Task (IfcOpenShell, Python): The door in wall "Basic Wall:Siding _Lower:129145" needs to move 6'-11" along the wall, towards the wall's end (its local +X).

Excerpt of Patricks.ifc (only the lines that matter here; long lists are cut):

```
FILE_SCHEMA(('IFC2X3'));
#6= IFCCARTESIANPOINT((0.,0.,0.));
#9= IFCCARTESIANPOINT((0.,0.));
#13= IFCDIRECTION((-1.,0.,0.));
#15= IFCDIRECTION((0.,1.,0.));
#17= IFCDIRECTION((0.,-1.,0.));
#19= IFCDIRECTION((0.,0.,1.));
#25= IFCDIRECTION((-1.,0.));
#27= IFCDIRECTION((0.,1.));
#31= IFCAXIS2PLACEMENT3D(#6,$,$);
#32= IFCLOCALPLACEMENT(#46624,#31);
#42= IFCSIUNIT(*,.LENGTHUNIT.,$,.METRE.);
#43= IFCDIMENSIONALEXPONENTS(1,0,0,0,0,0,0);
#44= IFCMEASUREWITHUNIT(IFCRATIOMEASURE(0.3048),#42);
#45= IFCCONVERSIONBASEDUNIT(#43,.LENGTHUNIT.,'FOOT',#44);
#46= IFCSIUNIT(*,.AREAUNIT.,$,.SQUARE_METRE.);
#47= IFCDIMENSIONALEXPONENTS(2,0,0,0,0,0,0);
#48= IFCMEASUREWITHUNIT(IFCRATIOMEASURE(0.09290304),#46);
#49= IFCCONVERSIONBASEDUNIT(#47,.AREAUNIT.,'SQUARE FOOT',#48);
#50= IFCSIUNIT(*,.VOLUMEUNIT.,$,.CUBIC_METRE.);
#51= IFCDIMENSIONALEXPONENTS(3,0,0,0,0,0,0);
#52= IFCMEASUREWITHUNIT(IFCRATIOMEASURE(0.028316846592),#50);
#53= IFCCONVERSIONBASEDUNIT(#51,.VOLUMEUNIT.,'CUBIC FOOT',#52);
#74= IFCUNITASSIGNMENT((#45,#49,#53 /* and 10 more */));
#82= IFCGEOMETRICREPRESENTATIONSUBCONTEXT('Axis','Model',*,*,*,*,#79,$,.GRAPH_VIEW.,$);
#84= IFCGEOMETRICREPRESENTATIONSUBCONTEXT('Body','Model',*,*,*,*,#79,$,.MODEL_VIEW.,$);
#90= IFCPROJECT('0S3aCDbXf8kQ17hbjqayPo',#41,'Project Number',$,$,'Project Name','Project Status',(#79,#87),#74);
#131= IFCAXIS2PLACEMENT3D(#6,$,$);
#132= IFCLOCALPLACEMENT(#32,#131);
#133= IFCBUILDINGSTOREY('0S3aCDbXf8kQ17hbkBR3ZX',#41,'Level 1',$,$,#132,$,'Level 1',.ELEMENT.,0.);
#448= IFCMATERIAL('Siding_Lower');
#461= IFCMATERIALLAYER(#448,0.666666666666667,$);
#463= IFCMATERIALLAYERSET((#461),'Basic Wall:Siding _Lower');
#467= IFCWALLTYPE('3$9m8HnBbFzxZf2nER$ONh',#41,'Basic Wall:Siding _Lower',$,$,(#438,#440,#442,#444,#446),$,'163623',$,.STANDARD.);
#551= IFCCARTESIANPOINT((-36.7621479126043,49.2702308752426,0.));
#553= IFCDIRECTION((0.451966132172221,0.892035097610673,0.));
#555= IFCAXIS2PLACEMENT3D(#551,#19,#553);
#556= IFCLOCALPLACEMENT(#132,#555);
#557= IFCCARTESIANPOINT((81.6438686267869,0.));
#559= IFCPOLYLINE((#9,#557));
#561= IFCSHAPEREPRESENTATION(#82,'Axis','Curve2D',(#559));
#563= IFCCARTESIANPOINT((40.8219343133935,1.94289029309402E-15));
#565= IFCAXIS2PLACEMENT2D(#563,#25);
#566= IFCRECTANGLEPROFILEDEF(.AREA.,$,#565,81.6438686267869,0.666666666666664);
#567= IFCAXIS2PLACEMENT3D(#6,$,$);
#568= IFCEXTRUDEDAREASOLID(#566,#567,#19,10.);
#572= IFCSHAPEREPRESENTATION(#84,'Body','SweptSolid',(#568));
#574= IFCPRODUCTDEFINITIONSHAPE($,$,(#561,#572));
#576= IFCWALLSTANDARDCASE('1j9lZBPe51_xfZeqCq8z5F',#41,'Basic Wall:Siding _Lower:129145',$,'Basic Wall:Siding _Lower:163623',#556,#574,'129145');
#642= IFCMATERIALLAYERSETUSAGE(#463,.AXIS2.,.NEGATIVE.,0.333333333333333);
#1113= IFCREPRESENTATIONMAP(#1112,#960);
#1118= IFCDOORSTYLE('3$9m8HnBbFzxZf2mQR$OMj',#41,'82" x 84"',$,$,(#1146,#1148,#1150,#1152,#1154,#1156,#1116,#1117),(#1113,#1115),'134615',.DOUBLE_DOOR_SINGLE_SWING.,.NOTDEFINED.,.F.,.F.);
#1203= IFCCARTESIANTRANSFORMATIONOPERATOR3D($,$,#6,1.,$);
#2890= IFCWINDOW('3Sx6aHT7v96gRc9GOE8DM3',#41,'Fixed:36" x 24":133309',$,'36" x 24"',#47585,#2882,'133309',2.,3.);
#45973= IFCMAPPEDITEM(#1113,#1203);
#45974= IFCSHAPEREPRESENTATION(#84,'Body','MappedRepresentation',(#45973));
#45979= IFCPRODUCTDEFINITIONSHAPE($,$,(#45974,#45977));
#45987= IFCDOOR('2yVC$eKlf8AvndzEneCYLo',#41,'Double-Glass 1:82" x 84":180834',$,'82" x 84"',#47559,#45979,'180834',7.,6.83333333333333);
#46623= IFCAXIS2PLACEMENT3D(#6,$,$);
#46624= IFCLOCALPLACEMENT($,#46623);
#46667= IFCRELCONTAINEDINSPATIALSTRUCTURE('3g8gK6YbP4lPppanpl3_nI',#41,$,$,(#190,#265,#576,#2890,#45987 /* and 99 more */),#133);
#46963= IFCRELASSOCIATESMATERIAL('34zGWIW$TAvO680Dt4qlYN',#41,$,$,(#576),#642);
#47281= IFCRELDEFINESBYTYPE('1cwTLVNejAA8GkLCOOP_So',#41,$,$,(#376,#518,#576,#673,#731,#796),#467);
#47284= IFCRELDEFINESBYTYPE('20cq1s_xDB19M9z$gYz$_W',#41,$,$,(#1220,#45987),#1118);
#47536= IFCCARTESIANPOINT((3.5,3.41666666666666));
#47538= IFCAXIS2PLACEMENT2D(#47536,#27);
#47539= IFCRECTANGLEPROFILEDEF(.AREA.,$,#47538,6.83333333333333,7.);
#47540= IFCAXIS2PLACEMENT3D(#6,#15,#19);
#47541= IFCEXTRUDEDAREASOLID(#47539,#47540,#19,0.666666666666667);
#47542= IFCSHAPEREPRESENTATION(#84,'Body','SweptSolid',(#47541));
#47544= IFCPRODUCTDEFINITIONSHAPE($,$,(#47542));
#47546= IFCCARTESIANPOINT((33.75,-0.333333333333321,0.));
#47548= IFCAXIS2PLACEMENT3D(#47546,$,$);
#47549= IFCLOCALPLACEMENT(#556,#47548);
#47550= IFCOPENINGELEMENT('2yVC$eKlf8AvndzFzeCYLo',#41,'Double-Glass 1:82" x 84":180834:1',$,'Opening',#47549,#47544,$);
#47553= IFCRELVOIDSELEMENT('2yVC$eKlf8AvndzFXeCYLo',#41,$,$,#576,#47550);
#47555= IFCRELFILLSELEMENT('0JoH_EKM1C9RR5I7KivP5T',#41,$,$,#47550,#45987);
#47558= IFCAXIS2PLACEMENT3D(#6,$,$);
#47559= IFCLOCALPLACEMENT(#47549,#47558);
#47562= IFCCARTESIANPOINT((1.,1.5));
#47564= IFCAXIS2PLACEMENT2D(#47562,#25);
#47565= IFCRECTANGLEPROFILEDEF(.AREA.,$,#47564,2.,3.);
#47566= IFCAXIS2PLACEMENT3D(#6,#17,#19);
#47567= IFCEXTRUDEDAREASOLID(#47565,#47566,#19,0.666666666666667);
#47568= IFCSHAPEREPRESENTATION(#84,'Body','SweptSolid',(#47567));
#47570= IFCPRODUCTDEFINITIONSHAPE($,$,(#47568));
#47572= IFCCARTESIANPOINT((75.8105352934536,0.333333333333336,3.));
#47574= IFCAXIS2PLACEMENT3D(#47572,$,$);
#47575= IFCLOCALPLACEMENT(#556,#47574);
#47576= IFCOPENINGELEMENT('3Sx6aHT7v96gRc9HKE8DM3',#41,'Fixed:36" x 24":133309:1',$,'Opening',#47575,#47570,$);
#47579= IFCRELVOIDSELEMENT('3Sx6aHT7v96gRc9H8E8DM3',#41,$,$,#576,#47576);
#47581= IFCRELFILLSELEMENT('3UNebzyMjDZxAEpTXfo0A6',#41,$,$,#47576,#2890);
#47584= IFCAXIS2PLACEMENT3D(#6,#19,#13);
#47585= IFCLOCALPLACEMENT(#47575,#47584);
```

```python
import ifcopenshell
import ifcopenshell.api.geometry
import ifcopenshell.util.placement
import ifcopenshell.util.unit

model = ifcopenshell.open("Patricks.ifc")
unit_scale = ifcopenshell.util.unit.calculate_unit_scale(model)

door = model.by_guid("2yVC$eKlf8AvndzEneCYLo")
opening = door.FillsVoids[0].RelatingOpeningElement
wall = opening.VoidsElements[0].RelatingBuildingElement

wall_matrix = ifcopenshell.util.placement.get_local_placement(wall.ObjectPlacement)
shift = wall_matrix[:3, 0] * 83 * 0.0254 / unit_scale
before = ifcopenshell.util.placement.get_local_placement(door.ObjectPlacement)[:3, 3].copy()

# The door is placed relative to its opening, so it follows when the opening moves.
matrix = ifcopenshell.util.placement.get_local_placement(opening.ObjectPlacement)
matrix[:3, 3] += shift
ifcopenshell.api.geometry.edit_object_placement(
    model, product=opening, matrix=matrix, is_si=False, should_transform_children=True
)

after = ifcopenshell.util.placement.get_local_placement(door.ObjectPlacement)[:3, 3]
print("door moved by", (after - before).round(3) + 0.0)

model.write("Patricks_updated.ifc")
```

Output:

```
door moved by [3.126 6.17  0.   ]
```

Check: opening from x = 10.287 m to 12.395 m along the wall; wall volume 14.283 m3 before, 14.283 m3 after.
